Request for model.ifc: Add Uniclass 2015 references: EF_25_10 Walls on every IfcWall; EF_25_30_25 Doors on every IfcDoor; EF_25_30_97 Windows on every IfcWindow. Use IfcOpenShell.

First a look at what the model holds.

```python
import ifcopenshell

model = ifcopenshell.open("model.ifc")
print(model.schema)
print("classifications:", [c.Name for c in model.by_type("IfcClassification")])
for ifc_class in ("IfcDoor", "IfcRoof", "IfcStair", "IfcWall", "IfcWindow"):
    print(ifc_class, len(model.by_type(ifc_class)))
```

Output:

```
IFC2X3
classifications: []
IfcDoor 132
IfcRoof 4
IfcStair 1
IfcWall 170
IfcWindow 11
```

```python
import ifcopenshell
import ifcopenshell.api.classification

model = ifcopenshell.open("model.ifc")

# IFC2X3 requires Source and Edition and has no link from the project to the system.
system = model.create_entity("IfcClassification", Source="NBS", Edition="2015", Name="Uniclass 2015")

codes = {
    "IfcWall": ("EF_25_10", "Walls"),
    "IfcDoor": ("EF_25_30_25", "Doors"),
    "IfcWindow": ("EF_25_30_97", "Windows"),
}
for ifc_class, (code, name) in codes.items():
    products = model.by_type(ifc_class)
    ifcopenshell.api.classification.add_reference(
        model, products=products, classification=system, identification=code, name=name
    )
    print(code, len(products))

model.write("model-out.ifc")
```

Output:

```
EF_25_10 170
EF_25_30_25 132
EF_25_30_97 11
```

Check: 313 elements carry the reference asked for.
